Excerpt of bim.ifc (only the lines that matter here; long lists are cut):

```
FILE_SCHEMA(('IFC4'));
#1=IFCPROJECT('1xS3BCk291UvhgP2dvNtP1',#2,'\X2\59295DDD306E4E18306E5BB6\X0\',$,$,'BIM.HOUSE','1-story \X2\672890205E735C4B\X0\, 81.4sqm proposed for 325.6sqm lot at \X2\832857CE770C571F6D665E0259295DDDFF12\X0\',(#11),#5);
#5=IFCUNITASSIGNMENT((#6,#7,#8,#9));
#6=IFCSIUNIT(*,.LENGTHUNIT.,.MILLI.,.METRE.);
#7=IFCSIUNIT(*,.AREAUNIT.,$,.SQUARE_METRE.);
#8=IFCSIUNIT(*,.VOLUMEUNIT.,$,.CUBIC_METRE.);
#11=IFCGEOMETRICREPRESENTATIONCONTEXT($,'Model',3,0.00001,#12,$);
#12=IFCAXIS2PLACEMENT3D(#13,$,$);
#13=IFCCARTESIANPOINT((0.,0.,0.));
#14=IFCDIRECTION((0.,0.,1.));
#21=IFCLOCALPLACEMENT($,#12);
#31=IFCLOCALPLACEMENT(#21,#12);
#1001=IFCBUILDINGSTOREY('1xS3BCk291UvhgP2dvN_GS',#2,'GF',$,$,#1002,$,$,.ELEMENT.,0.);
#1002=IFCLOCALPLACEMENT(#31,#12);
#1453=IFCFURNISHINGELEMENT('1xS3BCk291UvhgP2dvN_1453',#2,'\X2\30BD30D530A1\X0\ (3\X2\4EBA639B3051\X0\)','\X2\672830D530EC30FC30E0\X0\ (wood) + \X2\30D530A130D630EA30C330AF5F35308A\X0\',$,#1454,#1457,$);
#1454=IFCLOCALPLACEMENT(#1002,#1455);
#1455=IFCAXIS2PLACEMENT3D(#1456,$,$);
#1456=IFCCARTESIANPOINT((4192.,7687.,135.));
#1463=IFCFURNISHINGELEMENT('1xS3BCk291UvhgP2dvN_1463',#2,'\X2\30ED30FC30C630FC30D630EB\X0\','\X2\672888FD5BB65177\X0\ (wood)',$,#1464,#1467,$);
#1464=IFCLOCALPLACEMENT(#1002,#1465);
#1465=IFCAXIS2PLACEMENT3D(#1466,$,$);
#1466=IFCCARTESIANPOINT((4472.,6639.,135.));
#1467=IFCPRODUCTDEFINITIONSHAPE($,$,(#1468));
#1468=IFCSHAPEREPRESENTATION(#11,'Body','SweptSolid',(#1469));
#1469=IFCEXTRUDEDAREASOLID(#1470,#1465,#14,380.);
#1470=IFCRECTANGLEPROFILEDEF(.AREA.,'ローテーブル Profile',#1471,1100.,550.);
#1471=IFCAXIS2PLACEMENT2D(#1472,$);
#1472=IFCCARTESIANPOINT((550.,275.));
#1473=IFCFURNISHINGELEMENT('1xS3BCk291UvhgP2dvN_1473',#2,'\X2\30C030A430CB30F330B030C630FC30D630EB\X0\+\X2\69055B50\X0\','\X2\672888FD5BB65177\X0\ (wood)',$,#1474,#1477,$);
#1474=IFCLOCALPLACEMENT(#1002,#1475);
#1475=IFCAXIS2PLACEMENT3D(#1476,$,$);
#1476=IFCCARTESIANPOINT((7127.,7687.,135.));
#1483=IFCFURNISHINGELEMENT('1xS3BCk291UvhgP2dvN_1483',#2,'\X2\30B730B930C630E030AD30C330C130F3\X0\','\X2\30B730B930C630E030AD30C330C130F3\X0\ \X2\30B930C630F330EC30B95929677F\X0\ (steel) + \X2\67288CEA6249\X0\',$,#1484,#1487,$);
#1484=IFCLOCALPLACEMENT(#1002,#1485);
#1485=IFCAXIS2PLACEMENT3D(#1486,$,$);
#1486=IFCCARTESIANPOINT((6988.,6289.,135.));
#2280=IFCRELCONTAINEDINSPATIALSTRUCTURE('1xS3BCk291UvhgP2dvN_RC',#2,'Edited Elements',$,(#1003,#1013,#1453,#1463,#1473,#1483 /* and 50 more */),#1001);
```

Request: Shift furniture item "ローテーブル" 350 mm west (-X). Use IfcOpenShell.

```python
import ifcopenshell
import ifcopenshell.api.geometry
import ifcopenshell.util.placement

model = ifcopenshell.open("bim.ifc")

item = model.by_guid("1xS3BCk291UvhgP2dvN_1463")
matrix = ifcopenshell.util.placement.get_local_placement(item.ObjectPlacement)
matrix[0, 3] -= 350.0
ifcopenshell.api.geometry.edit_object_placement(model, product=item, matrix=matrix, is_si=False)

print(ifcopenshell.util.placement.get_local_placement(item.ObjectPlacement).round(3) + 0.0)

model.write("bim-out.ifc")
```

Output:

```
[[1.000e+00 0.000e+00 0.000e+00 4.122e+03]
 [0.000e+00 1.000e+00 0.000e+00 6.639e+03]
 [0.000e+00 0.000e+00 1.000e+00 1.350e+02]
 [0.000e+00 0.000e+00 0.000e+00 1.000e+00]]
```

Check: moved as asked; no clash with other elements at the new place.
